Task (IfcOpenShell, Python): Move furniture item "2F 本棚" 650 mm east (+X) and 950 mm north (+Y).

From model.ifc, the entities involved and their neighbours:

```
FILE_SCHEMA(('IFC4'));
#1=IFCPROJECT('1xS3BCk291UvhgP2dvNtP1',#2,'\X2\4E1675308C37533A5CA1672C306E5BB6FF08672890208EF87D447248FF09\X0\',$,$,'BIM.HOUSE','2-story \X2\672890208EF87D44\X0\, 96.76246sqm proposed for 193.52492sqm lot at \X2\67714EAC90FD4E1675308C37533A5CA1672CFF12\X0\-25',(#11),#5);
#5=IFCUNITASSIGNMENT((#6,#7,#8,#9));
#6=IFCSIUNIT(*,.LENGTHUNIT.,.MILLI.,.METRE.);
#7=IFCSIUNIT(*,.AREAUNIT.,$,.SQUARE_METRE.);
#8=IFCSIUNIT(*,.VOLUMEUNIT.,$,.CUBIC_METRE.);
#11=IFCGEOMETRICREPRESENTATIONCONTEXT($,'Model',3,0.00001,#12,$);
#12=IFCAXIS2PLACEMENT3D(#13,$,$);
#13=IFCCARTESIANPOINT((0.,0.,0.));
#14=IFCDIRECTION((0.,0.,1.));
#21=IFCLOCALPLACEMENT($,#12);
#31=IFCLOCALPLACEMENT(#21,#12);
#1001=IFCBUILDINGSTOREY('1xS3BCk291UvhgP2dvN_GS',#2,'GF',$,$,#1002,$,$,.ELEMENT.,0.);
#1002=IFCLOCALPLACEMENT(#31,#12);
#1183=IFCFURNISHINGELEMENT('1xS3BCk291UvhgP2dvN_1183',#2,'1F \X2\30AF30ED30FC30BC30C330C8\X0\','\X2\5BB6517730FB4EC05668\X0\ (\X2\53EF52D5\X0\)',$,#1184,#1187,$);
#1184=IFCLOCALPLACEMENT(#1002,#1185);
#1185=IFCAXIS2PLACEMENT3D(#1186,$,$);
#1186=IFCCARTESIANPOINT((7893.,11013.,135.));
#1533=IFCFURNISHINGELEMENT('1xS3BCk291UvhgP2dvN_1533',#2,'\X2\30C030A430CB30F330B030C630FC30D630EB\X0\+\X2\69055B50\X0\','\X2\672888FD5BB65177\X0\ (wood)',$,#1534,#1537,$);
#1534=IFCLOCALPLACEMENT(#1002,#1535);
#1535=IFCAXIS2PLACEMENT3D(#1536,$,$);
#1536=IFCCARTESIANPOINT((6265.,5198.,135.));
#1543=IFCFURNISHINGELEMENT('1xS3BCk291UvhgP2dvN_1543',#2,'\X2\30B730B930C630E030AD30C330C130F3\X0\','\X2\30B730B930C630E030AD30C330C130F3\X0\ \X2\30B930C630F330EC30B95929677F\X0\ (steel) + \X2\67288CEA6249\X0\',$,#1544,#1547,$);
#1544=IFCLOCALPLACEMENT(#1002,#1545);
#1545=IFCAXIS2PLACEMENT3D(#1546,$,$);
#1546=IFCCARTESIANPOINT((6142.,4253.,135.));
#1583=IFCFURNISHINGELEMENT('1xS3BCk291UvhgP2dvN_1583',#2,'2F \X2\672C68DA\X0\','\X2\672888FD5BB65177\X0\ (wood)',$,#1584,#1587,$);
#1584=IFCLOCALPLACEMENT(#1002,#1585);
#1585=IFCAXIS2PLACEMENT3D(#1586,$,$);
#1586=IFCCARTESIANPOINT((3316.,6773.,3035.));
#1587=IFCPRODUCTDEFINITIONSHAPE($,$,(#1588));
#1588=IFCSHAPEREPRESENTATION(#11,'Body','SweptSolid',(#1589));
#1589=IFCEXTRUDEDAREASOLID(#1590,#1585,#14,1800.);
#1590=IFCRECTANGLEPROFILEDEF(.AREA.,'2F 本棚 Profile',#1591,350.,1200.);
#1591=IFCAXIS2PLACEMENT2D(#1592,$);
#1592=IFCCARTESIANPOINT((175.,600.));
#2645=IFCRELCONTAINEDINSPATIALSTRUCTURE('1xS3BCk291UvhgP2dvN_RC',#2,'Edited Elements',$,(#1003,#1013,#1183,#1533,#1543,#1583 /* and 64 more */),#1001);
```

```python
import ifcopenshell
import ifcopenshell.api.geometry
import ifcopenshell.util.placement
import ifcopenshell.util.unit

model = ifcopenshell.open("model.ifc")
unit_scale = ifcopenshell.util.unit.calculate_unit_scale(model)

item = model.by_id(1583)
matrix = ifcopenshell.util.placement.get_local_placement(item.ObjectPlacement)
matrix[0, 3] += 0.65 / unit_scale
matrix[1, 3] += 0.95 / unit_scale
ifcopenshell.api.geometry.edit_object_placement(model, product=item, matrix=matrix, is_si=False)

print(ifcopenshell.util.placement.get_local_placement(item.ObjectPlacement).round(3) + 0.0)

model.write("model_updated.ifc")
```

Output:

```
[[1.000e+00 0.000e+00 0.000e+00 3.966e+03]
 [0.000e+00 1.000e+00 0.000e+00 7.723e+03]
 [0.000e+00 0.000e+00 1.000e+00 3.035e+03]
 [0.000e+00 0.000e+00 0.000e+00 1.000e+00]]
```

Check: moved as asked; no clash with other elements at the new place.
